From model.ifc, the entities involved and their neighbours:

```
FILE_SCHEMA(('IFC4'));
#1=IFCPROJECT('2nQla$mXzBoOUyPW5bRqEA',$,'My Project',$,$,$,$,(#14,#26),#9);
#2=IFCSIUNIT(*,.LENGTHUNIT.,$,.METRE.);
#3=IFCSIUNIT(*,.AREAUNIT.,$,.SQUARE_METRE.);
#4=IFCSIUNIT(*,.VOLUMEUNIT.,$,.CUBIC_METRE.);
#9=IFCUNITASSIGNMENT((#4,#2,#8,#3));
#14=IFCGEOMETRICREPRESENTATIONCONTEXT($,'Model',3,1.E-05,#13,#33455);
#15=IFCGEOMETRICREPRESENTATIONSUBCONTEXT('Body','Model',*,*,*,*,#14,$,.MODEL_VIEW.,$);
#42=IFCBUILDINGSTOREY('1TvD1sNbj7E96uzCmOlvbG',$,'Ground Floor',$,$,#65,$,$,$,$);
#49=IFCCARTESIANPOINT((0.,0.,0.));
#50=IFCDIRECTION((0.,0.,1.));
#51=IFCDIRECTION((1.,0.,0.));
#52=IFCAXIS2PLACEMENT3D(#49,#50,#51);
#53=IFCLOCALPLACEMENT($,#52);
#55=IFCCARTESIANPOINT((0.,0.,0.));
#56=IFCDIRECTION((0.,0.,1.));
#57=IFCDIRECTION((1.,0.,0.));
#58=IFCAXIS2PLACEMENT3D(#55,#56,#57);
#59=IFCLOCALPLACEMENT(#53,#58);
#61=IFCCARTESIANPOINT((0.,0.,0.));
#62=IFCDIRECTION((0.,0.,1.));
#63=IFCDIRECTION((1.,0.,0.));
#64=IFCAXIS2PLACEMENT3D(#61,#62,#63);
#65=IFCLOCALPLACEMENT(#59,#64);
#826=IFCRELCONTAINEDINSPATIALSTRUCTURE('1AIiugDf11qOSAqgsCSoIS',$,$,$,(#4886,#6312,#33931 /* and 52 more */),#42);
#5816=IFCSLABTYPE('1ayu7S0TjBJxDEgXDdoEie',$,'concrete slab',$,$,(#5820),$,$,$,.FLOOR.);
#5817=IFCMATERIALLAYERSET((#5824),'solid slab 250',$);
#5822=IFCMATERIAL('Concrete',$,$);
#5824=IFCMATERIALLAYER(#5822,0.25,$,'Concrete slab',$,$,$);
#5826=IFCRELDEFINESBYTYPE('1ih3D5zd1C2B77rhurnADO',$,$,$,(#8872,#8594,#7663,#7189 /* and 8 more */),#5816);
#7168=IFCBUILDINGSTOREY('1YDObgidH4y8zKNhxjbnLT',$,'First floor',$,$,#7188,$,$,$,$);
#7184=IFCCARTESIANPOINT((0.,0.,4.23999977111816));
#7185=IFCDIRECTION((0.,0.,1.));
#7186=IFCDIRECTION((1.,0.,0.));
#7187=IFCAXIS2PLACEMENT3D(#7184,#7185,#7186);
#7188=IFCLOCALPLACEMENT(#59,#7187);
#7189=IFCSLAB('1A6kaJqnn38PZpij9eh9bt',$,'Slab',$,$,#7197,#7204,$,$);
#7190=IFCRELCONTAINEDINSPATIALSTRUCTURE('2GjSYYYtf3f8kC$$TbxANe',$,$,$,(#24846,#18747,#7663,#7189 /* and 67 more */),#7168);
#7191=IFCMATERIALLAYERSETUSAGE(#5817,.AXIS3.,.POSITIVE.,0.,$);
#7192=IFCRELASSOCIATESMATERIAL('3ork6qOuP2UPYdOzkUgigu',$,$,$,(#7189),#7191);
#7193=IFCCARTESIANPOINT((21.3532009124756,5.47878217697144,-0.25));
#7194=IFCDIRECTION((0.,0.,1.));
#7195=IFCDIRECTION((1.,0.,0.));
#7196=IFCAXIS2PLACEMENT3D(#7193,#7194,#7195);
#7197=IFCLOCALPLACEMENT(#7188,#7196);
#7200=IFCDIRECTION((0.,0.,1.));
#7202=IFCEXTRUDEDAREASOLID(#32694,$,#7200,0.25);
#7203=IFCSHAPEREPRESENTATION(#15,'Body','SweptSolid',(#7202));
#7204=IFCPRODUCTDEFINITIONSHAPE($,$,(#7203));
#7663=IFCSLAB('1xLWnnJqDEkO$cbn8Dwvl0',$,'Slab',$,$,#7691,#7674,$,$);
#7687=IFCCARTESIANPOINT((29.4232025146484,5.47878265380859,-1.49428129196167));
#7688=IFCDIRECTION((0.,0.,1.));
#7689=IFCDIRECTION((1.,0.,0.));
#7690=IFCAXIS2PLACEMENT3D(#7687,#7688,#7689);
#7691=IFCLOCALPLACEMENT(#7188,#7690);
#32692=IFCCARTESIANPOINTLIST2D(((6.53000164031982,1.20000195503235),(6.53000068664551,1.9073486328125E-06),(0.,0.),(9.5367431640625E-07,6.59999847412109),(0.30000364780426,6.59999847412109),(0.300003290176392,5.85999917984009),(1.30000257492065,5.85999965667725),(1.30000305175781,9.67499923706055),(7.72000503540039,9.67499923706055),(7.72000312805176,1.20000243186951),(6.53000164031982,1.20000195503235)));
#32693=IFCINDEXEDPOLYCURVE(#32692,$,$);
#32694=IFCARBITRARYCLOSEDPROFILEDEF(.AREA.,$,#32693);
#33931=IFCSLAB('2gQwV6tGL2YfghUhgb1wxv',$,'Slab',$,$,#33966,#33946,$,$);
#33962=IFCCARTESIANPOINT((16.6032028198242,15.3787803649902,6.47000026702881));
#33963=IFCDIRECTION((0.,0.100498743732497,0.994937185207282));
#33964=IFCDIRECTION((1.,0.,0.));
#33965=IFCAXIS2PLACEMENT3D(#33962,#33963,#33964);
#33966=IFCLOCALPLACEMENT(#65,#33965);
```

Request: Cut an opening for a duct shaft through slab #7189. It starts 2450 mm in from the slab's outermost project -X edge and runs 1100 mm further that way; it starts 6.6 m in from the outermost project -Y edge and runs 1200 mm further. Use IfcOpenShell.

```python
import numpy as np
import ifcopenshell
import ifcopenshell.api.feature
import ifcopenshell.api.geometry
import ifcopenshell.api.root
import ifcopenshell.geom
import ifcopenshell.util.placement
import ifcopenshell.util.representation
import ifcopenshell.util.shape
import ifcopenshell.util.unit

model = ifcopenshell.open("model.ifc")
unit_scale = ifcopenshell.util.unit.calculate_unit_scale(model)
settings = ifcopenshell.geom.settings()


def volume(element):
    """Net volume in cubic metres, openings subtracted."""
    shape = ifcopenshell.geom.create_shape(settings, element)
    return ifcopenshell.util.shape.get_volume(shape.geometry)


slab = model.by_id(7189)
before = volume(slab)

# Extent in the slab's own axes, in metres. The edges named are its -X and -Y sides.
slab_shape = ifcopenshell.geom.create_shape(settings, slab)
vertices = ifcopenshell.util.shape.get_vertices(slab_shape.geometry)
x_min, y_min, bottom = vertices.min(axis=0)
top = vertices[:, 2].max()

opening = ifcopenshell.api.root.create_entity(model, ifc_class="IfcOpeningElement", name="Duct shaft opening", predefined_type="OPENING")
context = ifcopenshell.util.representation.get_context(model, "Model", "Body", "MODEL_VIEW")
width, depth = 1.1, 1.2
outline = [(0.0, 0.0), (width, 0.0), (width, depth), (0.0, depth), (0.0, 0.0)]
# Overshoot both faces by 50 mm so the cut is clean.
shape = ifcopenshell.api.geometry.add_slab_representation(
    model, context=context, depth=top - bottom + 0.1, polyline=outline
)
ifcopenshell.api.geometry.assign_representation(model, product=opening, representation=shape)

matrix = ifcopenshell.util.placement.get_local_placement(slab.ObjectPlacement)
matrix[:, 3] = matrix @ np.append(np.array([x_min + 2.45, y_min + 6.6, bottom - 0.05]) / unit_scale, 1.0)
ifcopenshell.api.geometry.edit_object_placement(model, product=opening, matrix=matrix, is_si=False)
ifcopenshell.api.feature.add_feature(model, feature=opening, element=slab)

after = volume(slab)

print(f"slab volume {before:.3f} -> {after:.3f} m3")

model.write("model_rev.ifc")
```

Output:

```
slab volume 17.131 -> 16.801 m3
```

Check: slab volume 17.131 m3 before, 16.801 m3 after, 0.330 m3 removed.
